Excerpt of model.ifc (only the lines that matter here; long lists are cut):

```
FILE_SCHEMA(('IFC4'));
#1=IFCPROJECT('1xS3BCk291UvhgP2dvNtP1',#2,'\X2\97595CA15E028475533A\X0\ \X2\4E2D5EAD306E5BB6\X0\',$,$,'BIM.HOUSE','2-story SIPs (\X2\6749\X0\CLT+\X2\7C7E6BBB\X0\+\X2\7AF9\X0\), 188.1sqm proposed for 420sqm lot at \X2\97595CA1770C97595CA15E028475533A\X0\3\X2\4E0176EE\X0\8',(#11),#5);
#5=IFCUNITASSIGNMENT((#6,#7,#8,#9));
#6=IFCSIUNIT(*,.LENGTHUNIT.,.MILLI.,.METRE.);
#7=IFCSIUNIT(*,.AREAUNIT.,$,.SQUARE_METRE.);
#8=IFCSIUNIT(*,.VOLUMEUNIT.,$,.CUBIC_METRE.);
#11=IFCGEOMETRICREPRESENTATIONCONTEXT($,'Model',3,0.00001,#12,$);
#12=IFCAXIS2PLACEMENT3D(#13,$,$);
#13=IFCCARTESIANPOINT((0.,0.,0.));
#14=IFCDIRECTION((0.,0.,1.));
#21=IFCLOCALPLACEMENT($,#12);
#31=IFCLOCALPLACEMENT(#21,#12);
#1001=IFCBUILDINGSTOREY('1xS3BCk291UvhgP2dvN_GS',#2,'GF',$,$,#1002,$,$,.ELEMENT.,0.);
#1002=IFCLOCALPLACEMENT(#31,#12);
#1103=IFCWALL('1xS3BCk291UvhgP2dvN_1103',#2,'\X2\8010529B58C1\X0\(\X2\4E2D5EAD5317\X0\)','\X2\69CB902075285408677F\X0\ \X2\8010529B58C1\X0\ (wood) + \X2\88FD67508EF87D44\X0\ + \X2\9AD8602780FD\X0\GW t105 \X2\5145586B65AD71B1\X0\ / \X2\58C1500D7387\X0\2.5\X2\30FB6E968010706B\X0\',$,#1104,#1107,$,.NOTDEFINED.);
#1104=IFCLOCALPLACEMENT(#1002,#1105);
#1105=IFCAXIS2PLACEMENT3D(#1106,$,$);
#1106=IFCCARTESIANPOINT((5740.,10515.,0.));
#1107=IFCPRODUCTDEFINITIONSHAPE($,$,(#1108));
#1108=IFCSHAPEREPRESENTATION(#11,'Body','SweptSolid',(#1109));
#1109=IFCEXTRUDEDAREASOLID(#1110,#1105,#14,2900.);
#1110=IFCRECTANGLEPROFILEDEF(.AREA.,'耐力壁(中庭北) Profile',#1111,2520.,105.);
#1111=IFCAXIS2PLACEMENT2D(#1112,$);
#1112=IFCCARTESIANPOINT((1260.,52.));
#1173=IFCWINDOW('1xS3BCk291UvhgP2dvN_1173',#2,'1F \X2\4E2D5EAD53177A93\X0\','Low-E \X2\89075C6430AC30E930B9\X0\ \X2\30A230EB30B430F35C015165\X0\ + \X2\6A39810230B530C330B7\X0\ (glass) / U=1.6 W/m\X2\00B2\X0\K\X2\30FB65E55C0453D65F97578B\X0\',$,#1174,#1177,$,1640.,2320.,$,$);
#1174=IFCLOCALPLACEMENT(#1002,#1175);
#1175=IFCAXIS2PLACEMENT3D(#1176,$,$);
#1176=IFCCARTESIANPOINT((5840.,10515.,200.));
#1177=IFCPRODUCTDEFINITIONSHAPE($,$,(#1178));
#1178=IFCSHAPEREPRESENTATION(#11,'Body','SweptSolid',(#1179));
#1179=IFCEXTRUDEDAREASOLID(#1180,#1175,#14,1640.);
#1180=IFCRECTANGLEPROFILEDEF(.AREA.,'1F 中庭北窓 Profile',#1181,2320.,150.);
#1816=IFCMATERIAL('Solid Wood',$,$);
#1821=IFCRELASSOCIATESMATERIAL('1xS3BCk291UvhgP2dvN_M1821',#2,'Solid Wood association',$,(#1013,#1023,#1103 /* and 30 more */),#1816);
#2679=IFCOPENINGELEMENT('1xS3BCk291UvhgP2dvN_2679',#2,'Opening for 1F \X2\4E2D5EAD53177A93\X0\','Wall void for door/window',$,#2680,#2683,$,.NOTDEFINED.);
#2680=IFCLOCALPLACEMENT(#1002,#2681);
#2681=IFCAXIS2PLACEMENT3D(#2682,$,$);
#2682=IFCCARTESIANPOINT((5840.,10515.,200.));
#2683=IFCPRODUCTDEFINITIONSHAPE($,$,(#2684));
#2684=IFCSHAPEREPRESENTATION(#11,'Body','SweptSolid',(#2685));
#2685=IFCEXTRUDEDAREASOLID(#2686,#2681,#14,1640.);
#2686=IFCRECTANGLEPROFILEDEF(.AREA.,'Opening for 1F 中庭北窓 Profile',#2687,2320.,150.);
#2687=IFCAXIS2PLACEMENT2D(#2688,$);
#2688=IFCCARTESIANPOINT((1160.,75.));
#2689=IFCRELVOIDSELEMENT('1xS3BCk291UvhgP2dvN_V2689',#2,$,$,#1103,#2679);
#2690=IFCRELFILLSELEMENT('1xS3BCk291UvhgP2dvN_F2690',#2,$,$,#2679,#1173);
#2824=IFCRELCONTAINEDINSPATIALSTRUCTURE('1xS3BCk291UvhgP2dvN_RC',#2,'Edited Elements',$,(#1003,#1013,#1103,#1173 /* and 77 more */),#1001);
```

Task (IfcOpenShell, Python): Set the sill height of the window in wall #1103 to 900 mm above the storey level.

```python
import numpy as np
import ifcopenshell
import ifcopenshell.api.geometry
import ifcopenshell.geom
import ifcopenshell.util.element
import ifcopenshell.util.placement
import ifcopenshell.util.shape
import ifcopenshell.util.unit

model = ifcopenshell.open("model.ifc")
unit_scale = ifcopenshell.util.unit.calculate_unit_scale(model)

window = model.by_guid("1xS3BCk291UvhgP2dvN_1173")
opening = window.FillsVoids[0].RelatingOpeningElement
storey = ifcopenshell.util.element.get_container(window, ifc_class="IfcBuildingStorey")
level = ifcopenshell.util.placement.get_local_placement(storey.ObjectPlacement)[2, 3]

# The opening's origin need not be at the sill, so measure its lowest point.
shape = ifcopenshell.geom.create_shape(ifcopenshell.geom.settings(), opening)
bottom = ifcopenshell.util.shape.get_shape_bottom_elevation(shape, shape.geometry) / unit_scale
dz = level + 0.9 / unit_scale - bottom

shift = np.array([0.0, 0.0, dz])
# The window is not placed relative to its opening, so move both.
for product in (opening, window):
    matrix = ifcopenshell.util.placement.get_local_placement(product.ObjectPlacement)
    matrix[:3, 3] += shift
    ifcopenshell.api.geometry.edit_object_placement(model, product=product, matrix=matrix, is_si=False)

print(f"moved by {dz * unit_scale:+.3f} m")

model.write("model-out.ifc")
```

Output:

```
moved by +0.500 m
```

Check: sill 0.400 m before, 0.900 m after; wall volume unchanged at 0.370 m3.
